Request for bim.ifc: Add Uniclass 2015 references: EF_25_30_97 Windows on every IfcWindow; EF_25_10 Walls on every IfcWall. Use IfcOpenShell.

First a look at what the model holds.

```python
import ifcopenshell

model = ifcopenshell.open("bim.ifc")
print(model.schema)
print("classifications:", [c.Name for c in model.by_type("IfcClassification")])
for ifc_class in ("IfcDoor", "IfcRoof", "IfcStair", "IfcWall", "IfcWindow"):
    print(ifc_class, len(model.by_type(ifc_class)))
```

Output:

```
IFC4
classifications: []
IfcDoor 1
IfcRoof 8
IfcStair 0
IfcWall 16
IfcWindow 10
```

```python
import ifcopenshell
import ifcopenshell.api.classification

model = ifcopenshell.open("bim.ifc")

system = ifcopenshell.api.classification.add_classification(model, classification="Uniclass 2015")

codes = {
    "IfcWindow": ("EF_25_30_97", "Windows"),
    "IfcWall": ("EF_25_10", "Walls"),
}
for ifc_class, (code, name) in codes.items():
    products = model.by_type(ifc_class)
    ifcopenshell.api.classification.add_reference(
        model, products=products, classification=system, identification=code, name=name
    )
    print(code, len(products))

model.write("bim-out.ifc")
```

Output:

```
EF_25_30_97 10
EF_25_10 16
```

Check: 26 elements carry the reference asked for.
